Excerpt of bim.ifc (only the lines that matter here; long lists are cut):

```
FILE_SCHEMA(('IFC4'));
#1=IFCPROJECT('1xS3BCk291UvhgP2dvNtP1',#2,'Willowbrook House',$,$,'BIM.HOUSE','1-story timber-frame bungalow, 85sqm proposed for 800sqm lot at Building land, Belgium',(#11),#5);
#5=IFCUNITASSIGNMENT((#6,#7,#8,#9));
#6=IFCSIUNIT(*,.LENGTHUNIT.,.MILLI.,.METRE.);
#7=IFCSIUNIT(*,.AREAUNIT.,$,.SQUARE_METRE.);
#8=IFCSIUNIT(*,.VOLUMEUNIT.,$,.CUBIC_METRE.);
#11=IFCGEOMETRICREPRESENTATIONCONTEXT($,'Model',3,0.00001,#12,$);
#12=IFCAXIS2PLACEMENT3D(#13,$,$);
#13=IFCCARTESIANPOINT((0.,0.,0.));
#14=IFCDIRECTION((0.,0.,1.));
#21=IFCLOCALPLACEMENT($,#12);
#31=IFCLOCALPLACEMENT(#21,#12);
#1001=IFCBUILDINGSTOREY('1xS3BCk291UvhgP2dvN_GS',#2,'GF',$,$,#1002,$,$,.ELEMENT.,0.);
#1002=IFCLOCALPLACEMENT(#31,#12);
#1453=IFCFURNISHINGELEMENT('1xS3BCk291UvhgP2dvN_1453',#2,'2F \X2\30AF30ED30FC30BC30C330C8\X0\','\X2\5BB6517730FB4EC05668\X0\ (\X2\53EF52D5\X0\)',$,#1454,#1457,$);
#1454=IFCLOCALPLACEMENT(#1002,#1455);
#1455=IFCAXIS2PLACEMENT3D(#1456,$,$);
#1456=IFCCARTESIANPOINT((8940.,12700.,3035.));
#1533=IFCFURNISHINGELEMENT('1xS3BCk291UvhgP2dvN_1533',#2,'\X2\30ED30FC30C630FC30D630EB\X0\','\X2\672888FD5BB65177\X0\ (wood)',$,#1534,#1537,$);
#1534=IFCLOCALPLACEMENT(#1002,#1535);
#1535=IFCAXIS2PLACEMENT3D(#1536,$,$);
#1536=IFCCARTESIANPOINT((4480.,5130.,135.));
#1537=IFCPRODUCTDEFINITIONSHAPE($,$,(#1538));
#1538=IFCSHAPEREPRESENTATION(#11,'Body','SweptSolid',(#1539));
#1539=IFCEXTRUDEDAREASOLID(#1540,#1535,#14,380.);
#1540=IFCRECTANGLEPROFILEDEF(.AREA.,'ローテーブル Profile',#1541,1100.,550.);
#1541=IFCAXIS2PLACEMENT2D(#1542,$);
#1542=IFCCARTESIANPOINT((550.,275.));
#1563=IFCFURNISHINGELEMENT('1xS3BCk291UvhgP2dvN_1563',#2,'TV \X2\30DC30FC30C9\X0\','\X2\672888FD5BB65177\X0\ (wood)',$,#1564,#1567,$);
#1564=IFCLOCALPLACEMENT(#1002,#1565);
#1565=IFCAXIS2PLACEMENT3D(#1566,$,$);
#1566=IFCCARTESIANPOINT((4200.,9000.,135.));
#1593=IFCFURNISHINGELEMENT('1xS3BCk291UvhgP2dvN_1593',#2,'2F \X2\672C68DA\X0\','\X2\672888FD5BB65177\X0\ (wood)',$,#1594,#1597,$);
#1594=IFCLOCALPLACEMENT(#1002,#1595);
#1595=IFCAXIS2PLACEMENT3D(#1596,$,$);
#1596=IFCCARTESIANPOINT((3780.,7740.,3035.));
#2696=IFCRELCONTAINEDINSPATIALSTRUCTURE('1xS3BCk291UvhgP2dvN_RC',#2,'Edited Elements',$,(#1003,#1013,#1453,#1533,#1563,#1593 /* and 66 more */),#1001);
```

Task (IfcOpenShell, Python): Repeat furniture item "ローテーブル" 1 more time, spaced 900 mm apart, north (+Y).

```python
import numpy as np
import ifcopenshell
import ifcopenshell.api.geometry
import ifcopenshell.api.root
import ifcopenshell.util.element
import ifcopenshell.util.placement
import ifcopenshell.util.unit

model = ifcopenshell.open("bim.ifc")
unit_scale = ifcopenshell.util.unit.calculate_unit_scale(model)


def reuse_history(source, copy):
    """copy_class also copies each property set's owner history, people and application; keep the originals."""
    for rel in copy.IsDefinedBy:
        if rel.is_a("IfcRelDefinesByProperties") and (history := rel.RelatingPropertyDefinition.OwnerHistory):
            rel.RelatingPropertyDefinition.OwnerHistory = source.OwnerHistory
            ifcopenshell.util.element.remove_deep2(model, history)


source = model.by_guid("1xS3BCk291UvhgP2dvN_1533")
base = ifcopenshell.util.placement.get_local_placement(source.ObjectPlacement)
step = np.array([0.0, 1.0, 0.0]) * 0.9 / unit_scale

for i in range(1, 2):
    copy = ifcopenshell.api.root.copy_class(model, product=source)
    copy.Representation = ifcopenshell.util.element.copy_deep(
        model, source.Representation, exclude=["IfcGeometricRepresentationContext", "IfcRepresentationMap"]
    )
    reuse_history(source, copy)
    matrix = base.copy()
    matrix[:3, 3] += i * step
    print("added at", matrix[:3, 3].round(3) + 0.0)
    ifcopenshell.api.geometry.edit_object_placement(model, product=copy, matrix=matrix, is_si=False)

model.write("bim_v2.ifc")
```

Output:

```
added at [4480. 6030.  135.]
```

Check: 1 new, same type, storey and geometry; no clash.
